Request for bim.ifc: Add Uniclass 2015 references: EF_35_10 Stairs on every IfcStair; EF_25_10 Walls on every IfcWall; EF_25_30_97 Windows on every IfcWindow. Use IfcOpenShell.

First a look at what the model holds.

```python
import ifcopenshell

model = ifcopenshell.open("bim.ifc")
print(model.schema)
print("classifications:", [c.Name for c in model.by_type("IfcClassification")])
for ifc_class in ("IfcDoor", "IfcRoof", "IfcStair", "IfcWall", "IfcWindow"):
    print(ifc_class, len(model.by_type(ifc_class)))
```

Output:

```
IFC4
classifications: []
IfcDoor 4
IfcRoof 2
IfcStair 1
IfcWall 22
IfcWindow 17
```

```python
import ifcopenshell
import ifcopenshell.api.classification

model = ifcopenshell.open("bim.ifc")

system = ifcopenshell.api.classification.add_classification(model, classification="Uniclass 2015")

codes = {
    "IfcStair": ("EF_35_10", "Stairs"),
    "IfcWall": ("EF_25_10", "Walls"),
    "IfcWindow": ("EF_25_30_97", "Windows"),
}
for ifc_class, (code, name) in codes.items():
    products = model.by_type(ifc_class)
    ifcopenshell.api.classification.add_reference(
        model, products=products, classification=system, identification=code, name=name
    )
    print(code, len(products))

model.write("bim-out.ifc")
```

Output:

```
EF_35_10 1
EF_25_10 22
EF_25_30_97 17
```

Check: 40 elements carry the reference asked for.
